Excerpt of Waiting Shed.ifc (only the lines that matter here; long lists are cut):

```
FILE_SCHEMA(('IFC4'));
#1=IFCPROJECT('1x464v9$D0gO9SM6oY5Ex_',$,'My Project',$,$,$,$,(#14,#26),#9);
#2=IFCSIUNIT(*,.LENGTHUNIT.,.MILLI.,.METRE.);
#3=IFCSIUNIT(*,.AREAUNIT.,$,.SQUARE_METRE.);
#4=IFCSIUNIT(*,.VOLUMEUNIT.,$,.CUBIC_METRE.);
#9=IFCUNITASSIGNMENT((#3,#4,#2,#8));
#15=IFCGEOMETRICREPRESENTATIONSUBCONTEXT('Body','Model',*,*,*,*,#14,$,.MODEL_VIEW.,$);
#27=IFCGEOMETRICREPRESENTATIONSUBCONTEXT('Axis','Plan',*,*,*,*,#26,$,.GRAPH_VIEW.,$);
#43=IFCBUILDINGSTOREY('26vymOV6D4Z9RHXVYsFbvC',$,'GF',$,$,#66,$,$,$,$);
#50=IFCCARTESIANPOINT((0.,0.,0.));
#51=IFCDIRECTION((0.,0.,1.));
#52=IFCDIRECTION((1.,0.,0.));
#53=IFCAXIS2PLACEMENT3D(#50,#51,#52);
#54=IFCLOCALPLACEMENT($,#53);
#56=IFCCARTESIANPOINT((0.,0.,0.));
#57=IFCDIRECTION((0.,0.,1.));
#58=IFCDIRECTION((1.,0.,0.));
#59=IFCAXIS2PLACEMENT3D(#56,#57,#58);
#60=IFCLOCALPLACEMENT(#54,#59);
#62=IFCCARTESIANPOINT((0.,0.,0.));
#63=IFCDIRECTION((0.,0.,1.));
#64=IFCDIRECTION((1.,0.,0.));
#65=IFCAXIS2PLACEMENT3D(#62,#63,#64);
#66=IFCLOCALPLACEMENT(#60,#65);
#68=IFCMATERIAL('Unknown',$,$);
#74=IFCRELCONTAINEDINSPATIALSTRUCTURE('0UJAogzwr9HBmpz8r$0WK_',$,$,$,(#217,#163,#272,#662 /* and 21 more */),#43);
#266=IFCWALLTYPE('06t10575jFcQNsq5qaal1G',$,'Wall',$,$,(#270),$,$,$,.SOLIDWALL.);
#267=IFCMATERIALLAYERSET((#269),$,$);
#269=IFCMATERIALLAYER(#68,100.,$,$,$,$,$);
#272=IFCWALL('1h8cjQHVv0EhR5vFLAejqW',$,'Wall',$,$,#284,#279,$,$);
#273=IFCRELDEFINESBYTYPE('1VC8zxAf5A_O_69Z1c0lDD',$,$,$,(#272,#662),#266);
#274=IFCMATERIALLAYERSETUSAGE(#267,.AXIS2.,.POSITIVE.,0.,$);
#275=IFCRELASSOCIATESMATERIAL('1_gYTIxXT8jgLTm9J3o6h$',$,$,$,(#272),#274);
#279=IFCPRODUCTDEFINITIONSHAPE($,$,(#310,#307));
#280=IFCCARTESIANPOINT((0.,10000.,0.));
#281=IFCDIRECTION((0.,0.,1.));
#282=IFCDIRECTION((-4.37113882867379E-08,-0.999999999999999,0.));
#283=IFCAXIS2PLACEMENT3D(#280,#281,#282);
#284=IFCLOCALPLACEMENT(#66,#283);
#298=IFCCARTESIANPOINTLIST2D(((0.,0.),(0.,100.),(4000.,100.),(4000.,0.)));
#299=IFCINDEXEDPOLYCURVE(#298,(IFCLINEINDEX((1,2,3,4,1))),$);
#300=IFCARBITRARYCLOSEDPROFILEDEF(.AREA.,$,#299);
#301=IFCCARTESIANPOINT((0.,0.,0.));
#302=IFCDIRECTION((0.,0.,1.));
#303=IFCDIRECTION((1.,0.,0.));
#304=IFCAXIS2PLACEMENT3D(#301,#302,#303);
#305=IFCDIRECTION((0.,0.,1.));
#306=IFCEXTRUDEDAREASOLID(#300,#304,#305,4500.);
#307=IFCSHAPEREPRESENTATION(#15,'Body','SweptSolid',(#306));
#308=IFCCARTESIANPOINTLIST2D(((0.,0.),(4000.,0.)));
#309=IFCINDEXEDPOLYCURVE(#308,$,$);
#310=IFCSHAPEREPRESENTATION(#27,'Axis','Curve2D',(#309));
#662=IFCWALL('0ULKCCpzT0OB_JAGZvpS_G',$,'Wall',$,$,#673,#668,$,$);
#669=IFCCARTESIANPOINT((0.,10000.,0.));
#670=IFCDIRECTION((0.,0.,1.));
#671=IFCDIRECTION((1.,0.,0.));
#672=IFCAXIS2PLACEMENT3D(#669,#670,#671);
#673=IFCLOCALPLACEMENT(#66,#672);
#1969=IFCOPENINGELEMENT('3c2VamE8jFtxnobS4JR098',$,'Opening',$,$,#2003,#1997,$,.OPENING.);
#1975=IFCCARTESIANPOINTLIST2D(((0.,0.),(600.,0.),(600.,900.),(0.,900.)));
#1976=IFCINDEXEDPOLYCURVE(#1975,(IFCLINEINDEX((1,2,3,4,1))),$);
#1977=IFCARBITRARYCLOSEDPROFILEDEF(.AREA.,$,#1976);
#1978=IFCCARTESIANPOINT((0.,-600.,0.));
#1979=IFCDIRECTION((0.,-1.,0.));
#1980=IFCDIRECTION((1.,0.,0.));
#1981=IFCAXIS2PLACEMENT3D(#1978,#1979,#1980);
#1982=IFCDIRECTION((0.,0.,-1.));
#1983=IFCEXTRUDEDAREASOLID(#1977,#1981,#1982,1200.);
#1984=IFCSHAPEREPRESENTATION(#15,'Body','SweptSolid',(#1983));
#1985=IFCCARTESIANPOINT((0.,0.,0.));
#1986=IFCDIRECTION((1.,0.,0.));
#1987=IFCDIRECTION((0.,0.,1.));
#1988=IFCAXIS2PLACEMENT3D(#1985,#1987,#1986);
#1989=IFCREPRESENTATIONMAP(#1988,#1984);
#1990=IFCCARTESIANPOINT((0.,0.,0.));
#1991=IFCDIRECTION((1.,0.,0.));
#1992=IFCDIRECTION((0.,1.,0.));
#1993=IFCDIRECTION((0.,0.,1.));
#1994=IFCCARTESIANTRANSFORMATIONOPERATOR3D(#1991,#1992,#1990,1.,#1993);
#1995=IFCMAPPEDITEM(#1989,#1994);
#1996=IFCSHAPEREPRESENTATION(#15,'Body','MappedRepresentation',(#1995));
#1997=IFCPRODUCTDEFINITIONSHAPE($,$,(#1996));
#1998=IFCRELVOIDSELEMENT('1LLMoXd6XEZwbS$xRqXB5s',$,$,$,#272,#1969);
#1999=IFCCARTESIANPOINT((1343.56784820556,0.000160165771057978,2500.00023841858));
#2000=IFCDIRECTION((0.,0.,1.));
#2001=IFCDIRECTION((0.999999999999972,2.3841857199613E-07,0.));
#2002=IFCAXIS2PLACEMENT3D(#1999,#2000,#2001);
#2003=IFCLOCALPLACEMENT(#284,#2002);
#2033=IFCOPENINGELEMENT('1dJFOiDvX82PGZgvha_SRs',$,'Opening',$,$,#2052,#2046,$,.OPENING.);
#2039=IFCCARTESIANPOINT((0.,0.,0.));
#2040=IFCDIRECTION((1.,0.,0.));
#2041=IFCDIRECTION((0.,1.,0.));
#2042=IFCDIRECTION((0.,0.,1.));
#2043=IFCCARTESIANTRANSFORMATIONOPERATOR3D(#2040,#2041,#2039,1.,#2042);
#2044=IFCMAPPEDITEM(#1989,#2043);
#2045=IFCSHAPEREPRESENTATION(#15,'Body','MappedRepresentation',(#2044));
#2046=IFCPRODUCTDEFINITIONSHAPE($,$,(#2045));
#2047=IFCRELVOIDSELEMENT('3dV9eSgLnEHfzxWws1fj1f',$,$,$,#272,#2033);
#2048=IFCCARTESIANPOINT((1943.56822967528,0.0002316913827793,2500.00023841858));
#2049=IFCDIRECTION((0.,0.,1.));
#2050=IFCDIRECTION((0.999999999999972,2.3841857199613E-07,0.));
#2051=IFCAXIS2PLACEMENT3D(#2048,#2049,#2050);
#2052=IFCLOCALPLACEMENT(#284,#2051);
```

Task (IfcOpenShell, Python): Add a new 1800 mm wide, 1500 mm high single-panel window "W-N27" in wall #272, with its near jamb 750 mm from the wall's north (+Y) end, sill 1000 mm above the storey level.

```python
import numpy as np
import ifcopenshell
import ifcopenshell.api.feature
import ifcopenshell.api.geometry
import ifcopenshell.api.root
import ifcopenshell.api.spatial
import ifcopenshell.geom
import ifcopenshell.util.element
import ifcopenshell.util.placement
import ifcopenshell.util.representation
import ifcopenshell.util.shape
import ifcopenshell.util.unit

model = ifcopenshell.open("Waiting Shed.ifc")
unit_scale = ifcopenshell.util.unit.calculate_unit_scale(model)
settings = ifcopenshell.geom.settings()


def volume(element):
    """Net volume in cubic metres, openings subtracted."""
    shape = ifcopenshell.geom.create_shape(settings, element)
    return ifcopenshell.util.shape.get_volume(shape.geometry)


wall = model.by_guid("1h8cjQHVv0EhR5vFLAejqW")
storey = ifcopenshell.util.element.get_container(wall, ifc_class="IfcBuildingStorey")
context = ifcopenshell.util.representation.get_context(model, "Model", "Body", "MODEL_VIEW")
before = volume(wall)

width, height, from_end, sill = 1.8, 1.5, 0.75, 1  # metres

# The wall runs along its own X axis, and the end named is its -X end.
wall_shape = ifcopenshell.geom.create_shape(settings, wall)
x, y, z = ifcopenshell.util.shape.get_vertices(wall_shape.geometry).T
start = x.min() + from_end
face, thickness = float(y.min()), float(y.max() - y.min())
wall_matrix = ifcopenshell.util.placement.get_local_placement(wall.ObjectPlacement)
level = ifcopenshell.util.placement.get_local_placement(storey.ObjectPlacement)[2, 3]


def in_wall(x, y):
    """Placement at x, y metres in the wall's axes, at sill height."""
    matrix = wall_matrix.copy()
    matrix[:, 3] = wall_matrix @ np.array([x / unit_scale, y / unit_scale, 0.0, 1.0])
    matrix[2, 3] = level + sill / unit_scale
    return matrix


# Opening: a box that overshoots both wall faces by 50 mm.
opening = ifcopenshell.api.root.create_entity(model, ifc_class="IfcOpeningElement", predefined_type="OPENING")
box = ifcopenshell.api.geometry.add_wall_representation(
    model, context=context, length=width, height=height, thickness=thickness + 0.1
)
ifcopenshell.api.geometry.assign_representation(model, product=opening, representation=box)
ifcopenshell.api.geometry.edit_object_placement(model, product=opening, matrix=in_wall(start, face - 0.05), is_si=False)
ifcopenshell.api.feature.add_feature(model, feature=opening, element=wall)

window = ifcopenshell.api.root.create_entity(model, ifc_class="IfcWindow", name="W-N27", predefined_type="WINDOW")
window.OverallWidth, window.OverallHeight = width / unit_scale, height / unit_scale
window.PartitioningType = "SINGLE_PANEL"
body = ifcopenshell.api.geometry.add_window_representation(
    model,
    context=context,
    overall_width=window.OverallWidth,
    overall_height=window.OverallHeight,
    partition_type="SINGLE_PANEL",
)
ifcopenshell.api.geometry.assign_representation(model, product=window, representation=body)
ifcopenshell.api.spatial.assign_container(model, products=[window], relating_structure=storey)
ifcopenshell.api.feature.add_filling(model, opening=opening, element=window)

# Centre the window in the wall's thickness.
ifcopenshell.api.geometry.edit_object_placement(model, product=window, matrix=in_wall(start, face), is_si=False)
window_shape = ifcopenshell.geom.create_shape(settings, window)
depth = ifcopenshell.util.shape.get_vertices(window_shape.geometry)[:, 1]
offset = face + thickness / 2 - (depth.min() + depth.max()) / 2
ifcopenshell.api.geometry.edit_object_placement(model, product=window, matrix=in_wall(start, offset), is_si=False)

after = volume(wall)

print(f"wall volume {before:.3f} -> {after:.3f} m3")

model.write("Waiting Shed_v2.ifc")
```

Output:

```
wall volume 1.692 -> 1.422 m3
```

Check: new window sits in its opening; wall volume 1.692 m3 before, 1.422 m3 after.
